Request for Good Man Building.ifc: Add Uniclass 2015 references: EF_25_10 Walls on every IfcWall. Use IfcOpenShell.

First a look at what the model holds.

```python
import ifcopenshell

model = ifcopenshell.open("Good Man Building.ifc")
print(model.schema)
print("classifications:", [c.Name for c in model.by_type("IfcClassification")])
for ifc_class in ("IfcDoor", "IfcRoof", "IfcStair", "IfcWall", "IfcWindow"):
    print(ifc_class, len(model.by_type(ifc_class)))
```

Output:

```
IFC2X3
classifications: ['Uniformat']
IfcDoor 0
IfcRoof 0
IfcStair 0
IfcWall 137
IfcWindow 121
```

```python
import ifcopenshell
import ifcopenshell.api.classification

model = ifcopenshell.open("Good Man Building.ifc")

# IFC2X3 requires Source and Edition and has no link from the project to the system.
system = model.create_entity("IfcClassification", Source="NBS", Edition="2015", Name="Uniclass 2015")

codes = {
    "IfcWall": ("EF_25_10", "Walls"),
}
for ifc_class, (code, name) in codes.items():
    products = model.by_type(ifc_class)
    ifcopenshell.api.classification.add_reference(
        model, products=products, classification=system, identification=code, name=name
    )
    print(code, len(products))

model.write("Good Man Building_v2.ifc")
```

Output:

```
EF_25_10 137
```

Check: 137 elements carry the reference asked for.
